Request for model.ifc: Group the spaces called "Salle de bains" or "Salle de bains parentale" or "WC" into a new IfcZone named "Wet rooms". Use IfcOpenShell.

First a look at what the model holds.

```python
import ifcopenshell

model = ifcopenshell.open("model.ifc")
print(model.schema)
seen = {}
for space in model.by_type("IfcSpace"):
    seen[space.LongName] = seen.get(space.LongName, 0) + 1
for name, count in sorted(seen.items(), key=str):
    print(count, "x", name)
print("zones:", [z.Name for z in model.by_type("IfcZone")][:20])
```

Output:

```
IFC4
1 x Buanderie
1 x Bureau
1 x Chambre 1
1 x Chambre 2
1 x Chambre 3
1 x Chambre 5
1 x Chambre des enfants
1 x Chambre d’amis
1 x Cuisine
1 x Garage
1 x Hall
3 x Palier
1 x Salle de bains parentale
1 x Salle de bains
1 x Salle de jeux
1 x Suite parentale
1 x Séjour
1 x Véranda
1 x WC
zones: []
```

```python
import ifcopenshell
import ifcopenshell.api.group
import ifcopenshell.api.root

model = ifcopenshell.open("model.ifc")

names = {"Salle de bains", "Salle de bains parentale", "WC"}
spaces = [s for s in model.by_type("IfcSpace") if s.LongName in names]

zone = ifcopenshell.api.root.create_entity(model, ifc_class="IfcZone", name="Wet rooms")
ifcopenshell.api.group.assign_group(model, products=spaces, group=zone)
print(len(spaces), "spaces in", zone.Name)

model.write("model-out.ifc")
```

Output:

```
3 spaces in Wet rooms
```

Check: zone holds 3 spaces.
